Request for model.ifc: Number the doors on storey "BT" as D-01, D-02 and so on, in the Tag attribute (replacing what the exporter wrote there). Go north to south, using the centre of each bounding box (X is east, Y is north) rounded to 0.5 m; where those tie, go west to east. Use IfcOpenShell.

First a look at what the model holds.

```python
import ifcopenshell
import ifcopenshell.util.element
import ifcopenshell.util.placement

model = ifcopenshell.open("model.ifc")
print(model.schema)
storey = next(s for s in model.by_type("IfcBuildingStorey") if s.Name == "BT")
doors = [e for e in ifcopenshell.util.element.get_decomposition(storey) if e.is_a("IfcDoor")]
for e in sorted(doors, key=lambda e: e.id()):
    origin = ifcopenshell.util.placement.get_local_placement(e.ObjectPlacement)[:3, 3]
    print(e.id(), e.Tag, e.Name, origin.round(2) + 0.0, sep=" | ")
```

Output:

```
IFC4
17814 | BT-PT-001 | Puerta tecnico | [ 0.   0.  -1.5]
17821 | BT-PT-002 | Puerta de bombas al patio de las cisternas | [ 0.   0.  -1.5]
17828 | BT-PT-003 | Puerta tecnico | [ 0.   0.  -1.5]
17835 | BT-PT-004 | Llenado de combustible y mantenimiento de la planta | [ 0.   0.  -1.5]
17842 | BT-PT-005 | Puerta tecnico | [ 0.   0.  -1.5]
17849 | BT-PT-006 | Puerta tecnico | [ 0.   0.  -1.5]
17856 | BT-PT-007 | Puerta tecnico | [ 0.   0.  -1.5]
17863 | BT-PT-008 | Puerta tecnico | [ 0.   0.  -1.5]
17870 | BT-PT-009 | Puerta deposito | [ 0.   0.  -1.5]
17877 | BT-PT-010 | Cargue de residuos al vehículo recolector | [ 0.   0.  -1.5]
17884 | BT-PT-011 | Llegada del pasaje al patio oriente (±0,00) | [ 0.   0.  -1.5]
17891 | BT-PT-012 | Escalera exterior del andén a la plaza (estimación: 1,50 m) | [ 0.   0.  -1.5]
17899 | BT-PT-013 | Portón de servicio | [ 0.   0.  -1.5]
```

```python
import ifcopenshell
import ifcopenshell.geom
import ifcopenshell.util.element
import ifcopenshell.util.shape

model = ifcopenshell.open("model.ifc")
settings = ifcopenshell.geom.settings()
settings.set("use-world-coords", True)


def centre(element):
    shape = ifcopenshell.geom.create_shape(settings, element)
    return ifcopenshell.util.shape.get_bbox_centroid(shape.geometry)


storey = next(s for s in model.by_type("IfcBuildingStorey") if s.Name == "BT")
doors = [e for e in ifcopenshell.util.element.get_decomposition(storey) if e.is_a("IfcDoor")]

# Insertion points can sit at a corner or the storey origin, so sort by the geometry (in metres).
centres = {e: centre(e) for e in doors}
doors.sort(key=lambda e: (-round(centres[e][1] / 0.5), centres[e][0]))

for i, e in enumerate(doors, start=1):
    number = f"D-{i:02d}"
    e.Tag = number
    print(e.id(), number)

model.write("model-out.ifc")
```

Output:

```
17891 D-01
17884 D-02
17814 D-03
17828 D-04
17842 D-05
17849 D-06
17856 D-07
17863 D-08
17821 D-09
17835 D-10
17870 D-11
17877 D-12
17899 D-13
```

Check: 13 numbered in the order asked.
